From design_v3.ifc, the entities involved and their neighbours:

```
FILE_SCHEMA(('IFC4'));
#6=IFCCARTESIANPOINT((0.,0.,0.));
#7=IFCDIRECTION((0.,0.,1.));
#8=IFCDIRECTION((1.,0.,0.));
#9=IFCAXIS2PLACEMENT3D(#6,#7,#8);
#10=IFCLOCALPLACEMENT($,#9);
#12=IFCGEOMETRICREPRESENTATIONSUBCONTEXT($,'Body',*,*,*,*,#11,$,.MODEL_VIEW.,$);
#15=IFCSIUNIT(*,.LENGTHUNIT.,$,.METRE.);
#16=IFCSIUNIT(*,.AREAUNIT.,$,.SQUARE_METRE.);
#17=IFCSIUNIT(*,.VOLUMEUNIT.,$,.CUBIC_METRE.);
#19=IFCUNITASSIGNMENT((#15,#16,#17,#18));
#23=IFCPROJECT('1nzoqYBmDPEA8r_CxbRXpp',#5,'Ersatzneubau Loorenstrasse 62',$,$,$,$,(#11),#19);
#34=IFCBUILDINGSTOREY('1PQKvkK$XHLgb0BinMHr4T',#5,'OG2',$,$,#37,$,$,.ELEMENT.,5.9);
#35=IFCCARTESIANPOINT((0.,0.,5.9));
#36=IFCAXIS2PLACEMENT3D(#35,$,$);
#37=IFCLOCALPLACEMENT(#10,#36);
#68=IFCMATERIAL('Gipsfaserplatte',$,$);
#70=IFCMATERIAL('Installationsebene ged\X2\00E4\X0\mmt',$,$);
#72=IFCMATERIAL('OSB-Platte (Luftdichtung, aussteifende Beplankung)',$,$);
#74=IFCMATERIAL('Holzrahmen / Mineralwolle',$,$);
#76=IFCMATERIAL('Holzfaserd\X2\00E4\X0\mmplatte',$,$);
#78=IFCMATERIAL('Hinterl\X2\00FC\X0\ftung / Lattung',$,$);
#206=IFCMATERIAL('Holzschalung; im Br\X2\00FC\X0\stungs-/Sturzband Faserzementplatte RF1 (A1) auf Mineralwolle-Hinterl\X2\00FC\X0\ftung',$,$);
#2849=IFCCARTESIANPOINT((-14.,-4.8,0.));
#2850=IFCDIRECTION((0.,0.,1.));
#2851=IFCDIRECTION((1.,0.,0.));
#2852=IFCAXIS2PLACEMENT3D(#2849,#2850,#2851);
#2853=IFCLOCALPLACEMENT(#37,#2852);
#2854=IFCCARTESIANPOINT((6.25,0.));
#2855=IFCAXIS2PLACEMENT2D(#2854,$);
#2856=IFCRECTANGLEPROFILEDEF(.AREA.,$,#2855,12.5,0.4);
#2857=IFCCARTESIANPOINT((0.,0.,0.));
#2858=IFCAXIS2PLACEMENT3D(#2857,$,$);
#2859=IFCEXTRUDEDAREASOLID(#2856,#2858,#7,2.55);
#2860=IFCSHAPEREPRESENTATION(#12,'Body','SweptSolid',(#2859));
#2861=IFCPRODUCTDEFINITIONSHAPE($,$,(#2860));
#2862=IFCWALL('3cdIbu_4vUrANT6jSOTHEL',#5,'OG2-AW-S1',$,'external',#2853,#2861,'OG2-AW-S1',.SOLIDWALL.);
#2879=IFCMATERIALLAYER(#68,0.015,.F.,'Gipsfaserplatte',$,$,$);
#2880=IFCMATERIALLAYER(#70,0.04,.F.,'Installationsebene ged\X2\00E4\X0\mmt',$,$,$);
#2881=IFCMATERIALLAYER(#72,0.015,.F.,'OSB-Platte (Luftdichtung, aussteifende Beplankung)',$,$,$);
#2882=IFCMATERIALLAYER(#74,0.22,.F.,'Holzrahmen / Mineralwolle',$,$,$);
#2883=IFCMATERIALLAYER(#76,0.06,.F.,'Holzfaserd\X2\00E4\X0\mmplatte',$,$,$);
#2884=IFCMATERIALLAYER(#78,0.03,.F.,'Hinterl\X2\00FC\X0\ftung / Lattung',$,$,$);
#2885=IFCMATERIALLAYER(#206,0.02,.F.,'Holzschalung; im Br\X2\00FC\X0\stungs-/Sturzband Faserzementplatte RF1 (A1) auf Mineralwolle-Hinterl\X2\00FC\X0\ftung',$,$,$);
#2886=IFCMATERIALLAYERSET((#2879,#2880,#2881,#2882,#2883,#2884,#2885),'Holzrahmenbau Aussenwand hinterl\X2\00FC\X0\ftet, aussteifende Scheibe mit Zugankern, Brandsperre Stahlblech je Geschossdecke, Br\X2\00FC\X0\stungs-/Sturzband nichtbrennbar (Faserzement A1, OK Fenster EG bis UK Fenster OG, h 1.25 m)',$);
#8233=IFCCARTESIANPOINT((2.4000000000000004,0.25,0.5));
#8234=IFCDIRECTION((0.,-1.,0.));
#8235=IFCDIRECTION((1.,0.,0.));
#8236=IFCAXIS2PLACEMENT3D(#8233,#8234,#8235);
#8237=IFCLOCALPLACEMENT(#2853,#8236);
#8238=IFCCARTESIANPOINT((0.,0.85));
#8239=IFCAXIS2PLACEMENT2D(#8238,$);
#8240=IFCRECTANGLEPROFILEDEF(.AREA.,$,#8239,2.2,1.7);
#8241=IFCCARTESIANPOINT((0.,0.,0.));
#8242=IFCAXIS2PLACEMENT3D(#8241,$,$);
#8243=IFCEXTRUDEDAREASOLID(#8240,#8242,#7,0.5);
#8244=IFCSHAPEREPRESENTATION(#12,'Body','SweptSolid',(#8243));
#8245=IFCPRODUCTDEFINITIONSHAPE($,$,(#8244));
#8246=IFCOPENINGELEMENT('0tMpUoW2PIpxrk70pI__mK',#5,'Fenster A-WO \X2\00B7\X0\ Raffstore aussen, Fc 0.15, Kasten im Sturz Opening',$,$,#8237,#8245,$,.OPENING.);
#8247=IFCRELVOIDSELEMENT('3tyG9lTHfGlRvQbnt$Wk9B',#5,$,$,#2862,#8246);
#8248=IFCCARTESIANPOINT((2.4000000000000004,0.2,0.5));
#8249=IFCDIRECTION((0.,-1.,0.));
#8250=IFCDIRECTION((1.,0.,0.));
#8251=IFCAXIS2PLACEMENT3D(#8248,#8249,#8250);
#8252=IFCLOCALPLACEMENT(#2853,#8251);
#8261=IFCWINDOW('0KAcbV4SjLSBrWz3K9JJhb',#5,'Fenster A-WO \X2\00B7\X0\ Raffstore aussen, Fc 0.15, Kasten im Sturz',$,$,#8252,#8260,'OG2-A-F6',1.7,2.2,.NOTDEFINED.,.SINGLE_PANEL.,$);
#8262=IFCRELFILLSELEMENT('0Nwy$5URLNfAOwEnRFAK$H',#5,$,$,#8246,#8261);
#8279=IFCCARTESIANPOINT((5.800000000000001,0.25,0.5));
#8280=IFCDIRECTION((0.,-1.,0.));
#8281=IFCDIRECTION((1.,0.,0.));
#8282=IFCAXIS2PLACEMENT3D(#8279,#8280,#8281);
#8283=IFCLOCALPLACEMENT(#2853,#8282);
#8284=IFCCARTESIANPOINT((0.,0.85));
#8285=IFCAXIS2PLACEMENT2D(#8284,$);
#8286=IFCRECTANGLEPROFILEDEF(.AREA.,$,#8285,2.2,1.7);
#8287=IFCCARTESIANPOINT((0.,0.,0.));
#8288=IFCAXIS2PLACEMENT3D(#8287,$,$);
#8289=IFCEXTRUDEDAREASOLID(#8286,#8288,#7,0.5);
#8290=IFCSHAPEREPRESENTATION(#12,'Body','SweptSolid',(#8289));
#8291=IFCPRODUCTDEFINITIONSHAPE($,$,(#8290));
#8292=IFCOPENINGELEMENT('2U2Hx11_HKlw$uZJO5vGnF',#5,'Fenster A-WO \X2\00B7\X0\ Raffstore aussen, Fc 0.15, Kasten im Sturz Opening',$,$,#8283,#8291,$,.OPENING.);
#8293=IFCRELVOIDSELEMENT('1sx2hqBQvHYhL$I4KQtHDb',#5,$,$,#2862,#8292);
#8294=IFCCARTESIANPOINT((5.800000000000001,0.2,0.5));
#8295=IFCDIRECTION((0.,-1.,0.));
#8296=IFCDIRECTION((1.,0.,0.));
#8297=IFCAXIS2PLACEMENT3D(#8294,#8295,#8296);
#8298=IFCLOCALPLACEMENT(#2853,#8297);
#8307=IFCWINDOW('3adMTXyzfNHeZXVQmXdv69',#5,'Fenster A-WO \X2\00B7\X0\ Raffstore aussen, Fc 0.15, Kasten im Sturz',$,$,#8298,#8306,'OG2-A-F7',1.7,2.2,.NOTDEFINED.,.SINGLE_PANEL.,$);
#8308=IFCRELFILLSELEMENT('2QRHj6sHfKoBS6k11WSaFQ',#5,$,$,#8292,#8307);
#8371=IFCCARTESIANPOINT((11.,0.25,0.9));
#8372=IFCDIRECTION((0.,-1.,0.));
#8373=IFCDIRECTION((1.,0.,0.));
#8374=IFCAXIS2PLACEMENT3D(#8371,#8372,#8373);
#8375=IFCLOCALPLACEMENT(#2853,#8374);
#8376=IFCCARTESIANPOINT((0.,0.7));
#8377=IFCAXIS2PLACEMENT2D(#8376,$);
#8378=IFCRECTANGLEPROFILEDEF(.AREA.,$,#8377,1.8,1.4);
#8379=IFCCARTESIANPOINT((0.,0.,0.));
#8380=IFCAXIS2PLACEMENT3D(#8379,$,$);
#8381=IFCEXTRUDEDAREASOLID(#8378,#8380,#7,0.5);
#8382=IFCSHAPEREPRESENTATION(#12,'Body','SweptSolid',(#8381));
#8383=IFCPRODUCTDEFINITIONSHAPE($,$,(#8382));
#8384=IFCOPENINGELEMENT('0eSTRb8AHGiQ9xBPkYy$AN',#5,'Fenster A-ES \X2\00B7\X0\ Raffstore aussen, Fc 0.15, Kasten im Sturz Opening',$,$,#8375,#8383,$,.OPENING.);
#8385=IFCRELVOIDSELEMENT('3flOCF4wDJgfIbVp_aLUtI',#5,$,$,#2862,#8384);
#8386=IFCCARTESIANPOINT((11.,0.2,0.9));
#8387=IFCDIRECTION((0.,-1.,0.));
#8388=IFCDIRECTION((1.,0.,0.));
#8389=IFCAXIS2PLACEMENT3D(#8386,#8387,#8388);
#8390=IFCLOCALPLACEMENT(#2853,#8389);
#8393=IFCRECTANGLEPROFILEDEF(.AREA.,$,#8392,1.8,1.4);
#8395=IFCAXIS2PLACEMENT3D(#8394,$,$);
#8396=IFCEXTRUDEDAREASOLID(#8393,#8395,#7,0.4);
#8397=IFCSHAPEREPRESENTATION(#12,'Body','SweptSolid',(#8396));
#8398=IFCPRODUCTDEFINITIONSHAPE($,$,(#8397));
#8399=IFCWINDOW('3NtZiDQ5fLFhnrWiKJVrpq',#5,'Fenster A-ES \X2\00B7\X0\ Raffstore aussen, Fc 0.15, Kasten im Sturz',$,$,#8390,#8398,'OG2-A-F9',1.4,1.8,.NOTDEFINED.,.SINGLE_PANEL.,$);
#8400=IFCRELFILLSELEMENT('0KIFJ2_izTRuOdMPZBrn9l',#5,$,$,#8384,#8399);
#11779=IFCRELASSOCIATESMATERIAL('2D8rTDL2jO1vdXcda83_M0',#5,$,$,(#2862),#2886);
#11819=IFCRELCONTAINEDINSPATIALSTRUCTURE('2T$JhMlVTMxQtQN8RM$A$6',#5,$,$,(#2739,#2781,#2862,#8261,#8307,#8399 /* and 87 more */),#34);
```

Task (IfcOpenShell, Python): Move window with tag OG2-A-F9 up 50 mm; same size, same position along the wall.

```python
import numpy as np
import ifcopenshell
import ifcopenshell.api.geometry
import ifcopenshell.util.placement
import ifcopenshell.util.unit

model = ifcopenshell.open("design_v3.ifc")
unit_scale = ifcopenshell.util.unit.calculate_unit_scale(model)

window = model.by_id(8399)
opening = window.FillsVoids[0].RelatingOpeningElement
dz = 0.05 / unit_scale

shift = np.array([0.0, 0.0, dz])
# The window is not placed relative to its opening, so move both.
for product in (opening, window):
    matrix = ifcopenshell.util.placement.get_local_placement(product.ObjectPlacement)
    matrix[:3, 3] += shift
    ifcopenshell.api.geometry.edit_object_placement(model, product=product, matrix=matrix, is_si=False)

print(f"moved by {dz * unit_scale:+.3f} m")

model.write("design_v3_rev.ifc")
```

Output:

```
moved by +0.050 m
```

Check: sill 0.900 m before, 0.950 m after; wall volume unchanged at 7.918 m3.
